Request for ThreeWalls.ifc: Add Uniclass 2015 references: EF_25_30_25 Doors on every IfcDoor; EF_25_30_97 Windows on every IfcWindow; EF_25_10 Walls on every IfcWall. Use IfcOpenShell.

First a look at what the model holds.

```python
import ifcopenshell

model = ifcopenshell.open("ThreeWalls.ifc")
print(model.schema)
print("classifications:", [c.Name for c in model.by_type("IfcClassification")])
for ifc_class in ("IfcDoor", "IfcRoof", "IfcStair", "IfcWall", "IfcWindow"):
    print(ifc_class, len(model.by_type(ifc_class)))
```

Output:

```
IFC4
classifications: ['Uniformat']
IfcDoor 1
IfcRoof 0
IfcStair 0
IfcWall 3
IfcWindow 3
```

```python
import ifcopenshell
import ifcopenshell.api.classification

model = ifcopenshell.open("ThreeWalls.ifc")

system = ifcopenshell.api.classification.add_classification(model, classification="Uniclass 2015")

codes = {
    "IfcDoor": ("EF_25_30_25", "Doors"),
    "IfcWindow": ("EF_25_30_97", "Windows"),
    "IfcWall": ("EF_25_10", "Walls"),
}
for ifc_class, (code, name) in codes.items():
    products = model.by_type(ifc_class)
    ifcopenshell.api.classification.add_reference(
        model, products=products, classification=system, identification=code, name=name
    )
    print(code, len(products))

model.write("ThreeWalls_v2.ifc")
```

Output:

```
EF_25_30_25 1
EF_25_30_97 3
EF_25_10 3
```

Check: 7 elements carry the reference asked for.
